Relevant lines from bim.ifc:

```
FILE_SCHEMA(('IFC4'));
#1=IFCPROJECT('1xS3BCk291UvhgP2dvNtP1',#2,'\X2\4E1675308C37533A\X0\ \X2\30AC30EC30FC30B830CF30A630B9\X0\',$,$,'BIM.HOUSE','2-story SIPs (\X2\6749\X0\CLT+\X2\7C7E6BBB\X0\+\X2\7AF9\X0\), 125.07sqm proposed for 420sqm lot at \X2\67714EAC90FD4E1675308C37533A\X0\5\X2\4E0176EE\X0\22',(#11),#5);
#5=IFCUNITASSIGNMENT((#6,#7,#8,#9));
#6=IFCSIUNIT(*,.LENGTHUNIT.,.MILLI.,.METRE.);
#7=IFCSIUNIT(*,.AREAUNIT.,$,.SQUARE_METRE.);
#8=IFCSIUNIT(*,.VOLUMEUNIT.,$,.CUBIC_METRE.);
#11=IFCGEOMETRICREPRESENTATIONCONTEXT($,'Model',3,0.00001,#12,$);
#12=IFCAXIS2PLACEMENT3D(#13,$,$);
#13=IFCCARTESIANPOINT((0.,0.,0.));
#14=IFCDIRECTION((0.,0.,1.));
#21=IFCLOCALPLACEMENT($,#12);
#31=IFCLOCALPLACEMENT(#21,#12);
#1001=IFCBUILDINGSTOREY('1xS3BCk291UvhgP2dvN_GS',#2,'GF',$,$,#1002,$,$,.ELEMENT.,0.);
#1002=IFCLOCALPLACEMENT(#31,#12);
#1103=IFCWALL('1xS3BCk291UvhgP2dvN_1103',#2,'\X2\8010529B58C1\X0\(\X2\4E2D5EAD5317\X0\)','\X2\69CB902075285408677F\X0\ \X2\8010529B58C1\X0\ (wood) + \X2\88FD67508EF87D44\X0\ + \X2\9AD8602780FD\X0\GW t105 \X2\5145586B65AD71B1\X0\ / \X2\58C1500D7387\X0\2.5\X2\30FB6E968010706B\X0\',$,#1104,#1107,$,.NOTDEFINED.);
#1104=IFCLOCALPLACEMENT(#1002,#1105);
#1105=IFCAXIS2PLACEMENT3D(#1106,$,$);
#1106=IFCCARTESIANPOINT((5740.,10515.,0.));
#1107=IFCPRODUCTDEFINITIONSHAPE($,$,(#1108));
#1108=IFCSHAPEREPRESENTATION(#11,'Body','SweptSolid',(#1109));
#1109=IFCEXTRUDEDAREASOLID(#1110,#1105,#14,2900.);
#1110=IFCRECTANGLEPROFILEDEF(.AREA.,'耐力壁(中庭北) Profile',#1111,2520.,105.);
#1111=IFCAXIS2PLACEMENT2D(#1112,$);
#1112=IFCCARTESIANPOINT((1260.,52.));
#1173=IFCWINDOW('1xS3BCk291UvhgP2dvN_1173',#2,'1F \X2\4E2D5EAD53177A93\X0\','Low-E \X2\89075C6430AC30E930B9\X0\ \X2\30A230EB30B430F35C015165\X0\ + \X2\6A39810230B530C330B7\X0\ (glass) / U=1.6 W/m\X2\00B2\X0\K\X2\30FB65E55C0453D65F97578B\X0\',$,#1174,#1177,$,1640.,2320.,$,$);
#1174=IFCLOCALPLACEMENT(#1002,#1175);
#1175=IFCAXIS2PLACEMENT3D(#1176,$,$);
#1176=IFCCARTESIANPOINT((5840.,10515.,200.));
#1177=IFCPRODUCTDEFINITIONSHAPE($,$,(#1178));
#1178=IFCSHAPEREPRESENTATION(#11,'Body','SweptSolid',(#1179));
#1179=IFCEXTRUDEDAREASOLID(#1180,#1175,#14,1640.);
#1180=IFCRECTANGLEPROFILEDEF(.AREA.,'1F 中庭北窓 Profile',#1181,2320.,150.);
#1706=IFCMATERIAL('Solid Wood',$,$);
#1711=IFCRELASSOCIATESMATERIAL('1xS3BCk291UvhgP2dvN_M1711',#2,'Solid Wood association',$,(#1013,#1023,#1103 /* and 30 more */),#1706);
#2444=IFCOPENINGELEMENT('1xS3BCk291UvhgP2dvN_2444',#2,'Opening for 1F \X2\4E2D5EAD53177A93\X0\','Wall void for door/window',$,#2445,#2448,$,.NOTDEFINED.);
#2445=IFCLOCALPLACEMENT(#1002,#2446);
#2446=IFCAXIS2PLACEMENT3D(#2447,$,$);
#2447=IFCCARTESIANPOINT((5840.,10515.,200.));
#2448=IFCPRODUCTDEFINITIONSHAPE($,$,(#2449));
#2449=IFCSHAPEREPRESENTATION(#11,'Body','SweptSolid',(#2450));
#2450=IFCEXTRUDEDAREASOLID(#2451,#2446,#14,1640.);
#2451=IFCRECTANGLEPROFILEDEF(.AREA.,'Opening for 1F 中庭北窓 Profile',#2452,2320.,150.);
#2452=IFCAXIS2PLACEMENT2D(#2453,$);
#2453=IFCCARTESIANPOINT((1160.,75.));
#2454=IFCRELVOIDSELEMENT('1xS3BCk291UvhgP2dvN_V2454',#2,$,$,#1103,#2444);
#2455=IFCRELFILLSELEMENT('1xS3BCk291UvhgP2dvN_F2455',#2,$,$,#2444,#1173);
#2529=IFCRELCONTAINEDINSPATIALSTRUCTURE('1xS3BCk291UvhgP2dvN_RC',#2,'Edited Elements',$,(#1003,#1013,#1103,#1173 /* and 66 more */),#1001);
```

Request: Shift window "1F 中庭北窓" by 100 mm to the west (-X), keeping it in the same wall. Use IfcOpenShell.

```python
import ifcopenshell
import ifcopenshell.api.geometry
import ifcopenshell.util.placement
import ifcopenshell.util.unit

model = ifcopenshell.open("bim.ifc")
unit_scale = ifcopenshell.util.unit.calculate_unit_scale(model)

window = model.by_guid("1xS3BCk291UvhgP2dvN_1173")
opening = window.FillsVoids[0].RelatingOpeningElement
wall = opening.VoidsElements[0].RelatingBuildingElement

wall_matrix = ifcopenshell.util.placement.get_local_placement(wall.ObjectPlacement)
shift = wall_matrix[:3, 0] * -0.1 / unit_scale
before = ifcopenshell.util.placement.get_local_placement(window.ObjectPlacement)[:3, 3].copy()

# The window is not placed relative to its opening, so move both.
for product in (opening, window):
    matrix = ifcopenshell.util.placement.get_local_placement(product.ObjectPlacement)
    matrix[:3, 3] += shift
    ifcopenshell.api.geometry.edit_object_placement(model, product=product, matrix=matrix, is_si=False)

after = ifcopenshell.util.placement.get_local_placement(window.ObjectPlacement)[:3, 3]
print("window moved by", (after - before).round(3) + 0.0)

model.write("bim_updated.ifc")
```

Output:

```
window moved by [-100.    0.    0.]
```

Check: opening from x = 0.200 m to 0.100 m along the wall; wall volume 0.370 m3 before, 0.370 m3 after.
